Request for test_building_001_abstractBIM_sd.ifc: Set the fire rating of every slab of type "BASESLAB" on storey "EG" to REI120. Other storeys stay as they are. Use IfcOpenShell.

First a look at what the model holds.

```python
import ifcopenshell
import ifcopenshell.util.element

model = ifcopenshell.open("test_building_001_abstractBIM_sd.ifc")
print(model.schema)
storey = next(s for s in model.by_type("IfcBuildingStorey") if s.Name == "EG")
slabs = [e for e in ifcopenshell.util.element.get_decomposition(storey) if e.is_a("IfcSlab")]
seen = {}
for e in slabs:
    element_type = ifcopenshell.util.element.get_type(e)
    key = (element_type.Name if element_type != e and element_type else None, ifcopenshell.util.element.get_pset(e, "Pset_SlabCommon", "FireRating"))
    seen[key] = seen.get(key, 0) + 1
for (name, value), count in sorted(seen.items(), key=str):
    print(count, "x", name, "|", value)
```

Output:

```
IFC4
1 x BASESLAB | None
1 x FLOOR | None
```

```python
import ifcopenshell
import ifcopenshell.api.pset
import ifcopenshell.util.element

model = ifcopenshell.open("test_building_001_abstractBIM_sd.ifc")

storey = next(s for s in model.by_type("IfcBuildingStorey") if s.Name == "EG")
slabs = [e for e in ifcopenshell.util.element.get_decomposition(storey) if e.is_a("IfcSlab")]

count = 0
for e in slabs:
    element_type = ifcopenshell.util.element.get_type(e)
    if element_type in (None, e) or element_type.Name != "BASESLAB":
        continue
    # add_pset returns the element's existing set when there is one.
    pset = ifcopenshell.api.pset.add_pset(model, product=e, name="Pset_SlabCommon")
    ifcopenshell.api.pset.edit_pset(model, pset=pset, properties={"FireRating": "REI120"})
    count += 1

print(count, "slabs updated")

model.write("test_building_001_abstractBIM_sd_edited.ifc")
```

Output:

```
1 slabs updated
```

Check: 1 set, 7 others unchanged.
